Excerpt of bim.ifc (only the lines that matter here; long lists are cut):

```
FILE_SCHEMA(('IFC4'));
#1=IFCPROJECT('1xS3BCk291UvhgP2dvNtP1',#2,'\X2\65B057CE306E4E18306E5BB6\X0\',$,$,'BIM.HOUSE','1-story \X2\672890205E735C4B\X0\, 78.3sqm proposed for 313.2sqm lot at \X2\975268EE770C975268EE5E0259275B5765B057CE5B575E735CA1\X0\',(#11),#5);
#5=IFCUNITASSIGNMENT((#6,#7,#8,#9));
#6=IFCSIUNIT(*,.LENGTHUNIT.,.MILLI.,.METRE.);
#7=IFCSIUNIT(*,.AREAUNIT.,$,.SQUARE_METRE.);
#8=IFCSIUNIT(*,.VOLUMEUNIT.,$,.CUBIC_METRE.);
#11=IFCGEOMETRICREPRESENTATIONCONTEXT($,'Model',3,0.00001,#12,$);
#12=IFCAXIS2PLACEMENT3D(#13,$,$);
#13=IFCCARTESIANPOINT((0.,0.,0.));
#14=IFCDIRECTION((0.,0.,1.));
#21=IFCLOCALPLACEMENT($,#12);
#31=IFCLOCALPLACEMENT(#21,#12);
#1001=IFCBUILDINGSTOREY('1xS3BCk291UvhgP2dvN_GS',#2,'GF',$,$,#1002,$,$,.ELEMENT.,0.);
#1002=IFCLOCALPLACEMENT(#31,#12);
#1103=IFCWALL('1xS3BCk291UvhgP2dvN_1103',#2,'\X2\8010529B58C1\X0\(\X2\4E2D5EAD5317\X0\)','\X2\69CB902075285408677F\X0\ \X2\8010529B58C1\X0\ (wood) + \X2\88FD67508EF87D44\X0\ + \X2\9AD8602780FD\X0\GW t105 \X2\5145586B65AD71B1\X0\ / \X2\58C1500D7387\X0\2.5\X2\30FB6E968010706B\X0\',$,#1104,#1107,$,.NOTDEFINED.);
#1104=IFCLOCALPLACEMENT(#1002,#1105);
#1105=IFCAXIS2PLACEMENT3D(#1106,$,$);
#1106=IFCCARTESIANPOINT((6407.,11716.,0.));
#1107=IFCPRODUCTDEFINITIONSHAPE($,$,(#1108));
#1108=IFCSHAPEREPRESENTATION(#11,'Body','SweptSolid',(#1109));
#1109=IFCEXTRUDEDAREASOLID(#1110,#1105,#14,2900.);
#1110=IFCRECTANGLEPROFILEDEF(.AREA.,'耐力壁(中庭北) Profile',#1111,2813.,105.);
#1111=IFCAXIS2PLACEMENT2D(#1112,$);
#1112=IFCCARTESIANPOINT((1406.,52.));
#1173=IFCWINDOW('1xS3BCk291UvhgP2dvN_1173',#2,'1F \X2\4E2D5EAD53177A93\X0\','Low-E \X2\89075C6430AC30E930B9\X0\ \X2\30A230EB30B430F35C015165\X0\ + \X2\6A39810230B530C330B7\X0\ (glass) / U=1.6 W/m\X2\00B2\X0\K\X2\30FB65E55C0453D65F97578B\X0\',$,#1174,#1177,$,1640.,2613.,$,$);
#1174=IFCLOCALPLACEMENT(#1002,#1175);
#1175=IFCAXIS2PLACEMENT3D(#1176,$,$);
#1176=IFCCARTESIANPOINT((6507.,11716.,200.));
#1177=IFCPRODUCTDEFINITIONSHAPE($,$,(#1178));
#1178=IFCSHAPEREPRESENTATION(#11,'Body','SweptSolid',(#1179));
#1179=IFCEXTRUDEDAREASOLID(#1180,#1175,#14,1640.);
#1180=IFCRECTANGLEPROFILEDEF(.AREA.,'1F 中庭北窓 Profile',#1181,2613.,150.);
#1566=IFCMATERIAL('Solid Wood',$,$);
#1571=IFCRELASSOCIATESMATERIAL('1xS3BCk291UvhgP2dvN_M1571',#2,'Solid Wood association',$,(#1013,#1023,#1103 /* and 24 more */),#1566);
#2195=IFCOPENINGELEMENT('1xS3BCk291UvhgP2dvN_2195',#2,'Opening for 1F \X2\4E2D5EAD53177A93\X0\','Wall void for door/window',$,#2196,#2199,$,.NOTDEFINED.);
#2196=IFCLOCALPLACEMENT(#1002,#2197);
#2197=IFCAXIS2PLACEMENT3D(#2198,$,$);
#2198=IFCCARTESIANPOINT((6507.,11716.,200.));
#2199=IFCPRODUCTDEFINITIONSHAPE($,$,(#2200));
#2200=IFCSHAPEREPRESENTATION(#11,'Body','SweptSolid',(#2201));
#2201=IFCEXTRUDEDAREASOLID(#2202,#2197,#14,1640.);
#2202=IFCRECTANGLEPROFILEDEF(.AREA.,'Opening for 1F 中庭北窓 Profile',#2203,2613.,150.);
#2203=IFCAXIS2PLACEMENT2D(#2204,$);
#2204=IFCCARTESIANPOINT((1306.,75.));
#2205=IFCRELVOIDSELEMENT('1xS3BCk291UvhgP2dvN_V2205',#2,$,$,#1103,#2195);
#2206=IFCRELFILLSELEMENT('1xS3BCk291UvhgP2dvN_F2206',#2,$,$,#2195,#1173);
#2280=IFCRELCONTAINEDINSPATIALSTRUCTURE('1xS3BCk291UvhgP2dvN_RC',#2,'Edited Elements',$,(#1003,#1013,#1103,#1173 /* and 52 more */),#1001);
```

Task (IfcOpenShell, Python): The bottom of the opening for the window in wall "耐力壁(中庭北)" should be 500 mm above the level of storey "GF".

```python
import numpy as np
import ifcopenshell
import ifcopenshell.api.geometry
import ifcopenshell.geom
import ifcopenshell.util.element
import ifcopenshell.util.placement
import ifcopenshell.util.shape
import ifcopenshell.util.unit

model = ifcopenshell.open("bim.ifc")
unit_scale = ifcopenshell.util.unit.calculate_unit_scale(model)

window = model.by_id(1173)
opening = window.FillsVoids[0].RelatingOpeningElement
storey = ifcopenshell.util.element.get_container(window, ifc_class="IfcBuildingStorey")
level = ifcopenshell.util.placement.get_local_placement(storey.ObjectPlacement)[2, 3]

# The opening's origin need not be at the sill, so measure its lowest point.
shape = ifcopenshell.geom.create_shape(ifcopenshell.geom.settings(), opening)
bottom = ifcopenshell.util.shape.get_shape_bottom_elevation(shape, shape.geometry) / unit_scale
dz = level + 500.0 - bottom

shift = np.array([0.0, 0.0, dz])
# The window is not placed relative to its opening, so move both.
for product in (opening, window):
    matrix = ifcopenshell.util.placement.get_local_placement(product.ObjectPlacement)
    matrix[:3, 3] += shift
    ifcopenshell.api.geometry.edit_object_placement(model, product=product, matrix=matrix, is_si=False)

print(f"moved by {dz * unit_scale:+.3f} m")

model.write("bim-out.ifc")
```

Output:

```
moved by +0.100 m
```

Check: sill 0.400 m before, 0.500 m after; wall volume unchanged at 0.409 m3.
